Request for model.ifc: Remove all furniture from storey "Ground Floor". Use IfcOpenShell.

First a look at what the model holds.

```python
import ifcopenshell
import ifcopenshell.util.element

model = ifcopenshell.open("model.ifc")
print(model.schema)
storey = next(s for s in model.by_type("IfcBuildingStorey") if s.Name == "Ground Floor")
furniture = [e for e in ifcopenshell.util.element.get_decomposition(storey) if e.is_a("IfcFurnishingElement")]
seen = {}
for e in furniture:
    element_type = ifcopenshell.util.element.get_type(e)
    name = element_type.Name if element_type not in (None, e) else None
    seen[name] = seen.get(name, 0) + 1
for name, count in sorted(seen.items(), key=str):
    print(count, "x", name)
```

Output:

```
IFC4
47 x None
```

```python
import ifcopenshell
import ifcopenshell.api.root
import ifcopenshell.util.element

model = ifcopenshell.open("model.ifc")

storey = next(s for s in model.by_type("IfcBuildingStorey") if s.Name == "Ground Floor")
furniture = [e for e in ifcopenshell.util.element.get_decomposition(storey) if e.is_a("IfcFurnishingElement")]

for e in furniture:
    ifcopenshell.api.root.remove_product(model, product=e)
print(len(furniture), "removed")

model.write("model-out.ifc")
```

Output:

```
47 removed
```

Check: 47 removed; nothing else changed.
